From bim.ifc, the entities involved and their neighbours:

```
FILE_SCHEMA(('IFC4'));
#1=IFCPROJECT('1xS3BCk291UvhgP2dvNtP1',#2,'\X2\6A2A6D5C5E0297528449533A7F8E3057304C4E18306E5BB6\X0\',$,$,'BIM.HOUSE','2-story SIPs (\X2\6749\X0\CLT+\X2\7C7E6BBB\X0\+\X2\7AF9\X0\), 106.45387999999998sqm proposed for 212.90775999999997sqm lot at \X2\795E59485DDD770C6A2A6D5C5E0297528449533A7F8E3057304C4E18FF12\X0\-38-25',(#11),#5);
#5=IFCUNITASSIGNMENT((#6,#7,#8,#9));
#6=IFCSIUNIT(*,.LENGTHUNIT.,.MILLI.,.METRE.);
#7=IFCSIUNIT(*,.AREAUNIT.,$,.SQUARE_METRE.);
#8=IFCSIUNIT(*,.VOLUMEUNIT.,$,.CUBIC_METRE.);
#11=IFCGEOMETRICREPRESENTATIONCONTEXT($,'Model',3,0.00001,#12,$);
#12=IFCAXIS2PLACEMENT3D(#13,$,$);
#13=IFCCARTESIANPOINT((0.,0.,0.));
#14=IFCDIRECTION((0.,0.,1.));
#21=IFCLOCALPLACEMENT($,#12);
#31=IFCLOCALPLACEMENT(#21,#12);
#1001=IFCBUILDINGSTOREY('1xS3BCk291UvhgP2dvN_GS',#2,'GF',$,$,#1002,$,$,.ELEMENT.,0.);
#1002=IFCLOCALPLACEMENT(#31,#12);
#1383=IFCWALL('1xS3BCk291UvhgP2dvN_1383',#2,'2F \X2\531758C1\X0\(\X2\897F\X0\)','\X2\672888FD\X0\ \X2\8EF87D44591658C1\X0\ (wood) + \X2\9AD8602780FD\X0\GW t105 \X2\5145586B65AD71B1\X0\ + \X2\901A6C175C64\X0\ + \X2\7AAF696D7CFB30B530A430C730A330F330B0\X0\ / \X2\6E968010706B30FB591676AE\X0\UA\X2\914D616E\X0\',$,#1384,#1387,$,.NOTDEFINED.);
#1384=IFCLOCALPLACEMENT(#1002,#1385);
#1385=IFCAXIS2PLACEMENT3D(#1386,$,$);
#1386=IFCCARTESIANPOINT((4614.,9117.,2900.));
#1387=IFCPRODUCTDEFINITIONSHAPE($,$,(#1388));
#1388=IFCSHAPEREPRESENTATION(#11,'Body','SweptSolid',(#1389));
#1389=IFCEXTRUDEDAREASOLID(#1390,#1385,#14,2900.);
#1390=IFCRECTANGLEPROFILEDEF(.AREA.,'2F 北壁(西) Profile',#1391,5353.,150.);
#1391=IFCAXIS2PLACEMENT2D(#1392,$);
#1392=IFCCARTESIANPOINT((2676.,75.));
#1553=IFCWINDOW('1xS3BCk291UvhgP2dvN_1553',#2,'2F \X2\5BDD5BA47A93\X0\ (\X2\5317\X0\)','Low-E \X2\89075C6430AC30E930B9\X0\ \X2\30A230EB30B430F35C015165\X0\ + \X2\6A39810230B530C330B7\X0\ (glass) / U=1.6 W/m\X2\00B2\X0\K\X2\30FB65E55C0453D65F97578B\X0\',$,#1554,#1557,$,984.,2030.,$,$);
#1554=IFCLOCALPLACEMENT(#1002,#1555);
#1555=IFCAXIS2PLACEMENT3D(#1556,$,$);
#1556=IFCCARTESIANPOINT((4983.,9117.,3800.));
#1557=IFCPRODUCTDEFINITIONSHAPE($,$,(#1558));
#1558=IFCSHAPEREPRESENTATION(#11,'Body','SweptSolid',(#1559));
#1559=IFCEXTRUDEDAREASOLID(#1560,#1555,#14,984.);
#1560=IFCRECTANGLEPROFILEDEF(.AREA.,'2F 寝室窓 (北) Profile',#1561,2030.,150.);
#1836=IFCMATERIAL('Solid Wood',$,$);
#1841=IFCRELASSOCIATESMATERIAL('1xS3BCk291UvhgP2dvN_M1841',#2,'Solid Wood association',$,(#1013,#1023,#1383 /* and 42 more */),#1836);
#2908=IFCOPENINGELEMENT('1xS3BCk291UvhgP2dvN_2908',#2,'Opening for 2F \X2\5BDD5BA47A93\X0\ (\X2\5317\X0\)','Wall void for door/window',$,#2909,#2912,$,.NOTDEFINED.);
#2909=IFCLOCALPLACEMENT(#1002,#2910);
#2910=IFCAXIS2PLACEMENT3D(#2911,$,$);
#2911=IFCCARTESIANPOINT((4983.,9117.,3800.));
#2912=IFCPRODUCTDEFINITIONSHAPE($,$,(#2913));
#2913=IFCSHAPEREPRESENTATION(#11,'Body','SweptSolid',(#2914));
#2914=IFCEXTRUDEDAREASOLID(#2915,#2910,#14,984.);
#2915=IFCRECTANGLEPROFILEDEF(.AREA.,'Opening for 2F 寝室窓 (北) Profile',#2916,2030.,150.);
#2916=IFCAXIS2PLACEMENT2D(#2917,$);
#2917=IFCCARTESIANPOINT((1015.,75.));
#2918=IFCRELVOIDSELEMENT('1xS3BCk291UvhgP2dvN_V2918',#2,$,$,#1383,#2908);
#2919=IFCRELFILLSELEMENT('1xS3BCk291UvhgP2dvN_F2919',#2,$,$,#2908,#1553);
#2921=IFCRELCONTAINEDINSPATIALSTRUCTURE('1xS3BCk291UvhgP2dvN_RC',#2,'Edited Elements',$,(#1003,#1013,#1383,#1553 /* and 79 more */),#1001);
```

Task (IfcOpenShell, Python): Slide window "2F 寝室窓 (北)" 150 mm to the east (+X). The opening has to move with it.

```python
import ifcopenshell
import ifcopenshell.api.geometry
import ifcopenshell.util.placement
import ifcopenshell.util.unit

model = ifcopenshell.open("bim.ifc")
unit_scale = ifcopenshell.util.unit.calculate_unit_scale(model)

window = model.by_id(1553)
opening = window.FillsVoids[0].RelatingOpeningElement
wall = opening.VoidsElements[0].RelatingBuildingElement

wall_matrix = ifcopenshell.util.placement.get_local_placement(wall.ObjectPlacement)
shift = wall_matrix[:3, 0] * 0.15 / unit_scale
before = ifcopenshell.util.placement.get_local_placement(window.ObjectPlacement)[:3, 3].copy()

# The window is not placed relative to its opening, so move both.
for product in (opening, window):
    matrix = ifcopenshell.util.placement.get_local_placement(product.ObjectPlacement)
    matrix[:3, 3] += shift
    ifcopenshell.api.geometry.edit_object_placement(model, product=product, matrix=matrix, is_si=False)

after = ifcopenshell.util.placement.get_local_placement(window.ObjectPlacement)[:3, 3]
print("window moved by", (after - before).round(3) + 0.0)

model.write("bim-out.ifc")
```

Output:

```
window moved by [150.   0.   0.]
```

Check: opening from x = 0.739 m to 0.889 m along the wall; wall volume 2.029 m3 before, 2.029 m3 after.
